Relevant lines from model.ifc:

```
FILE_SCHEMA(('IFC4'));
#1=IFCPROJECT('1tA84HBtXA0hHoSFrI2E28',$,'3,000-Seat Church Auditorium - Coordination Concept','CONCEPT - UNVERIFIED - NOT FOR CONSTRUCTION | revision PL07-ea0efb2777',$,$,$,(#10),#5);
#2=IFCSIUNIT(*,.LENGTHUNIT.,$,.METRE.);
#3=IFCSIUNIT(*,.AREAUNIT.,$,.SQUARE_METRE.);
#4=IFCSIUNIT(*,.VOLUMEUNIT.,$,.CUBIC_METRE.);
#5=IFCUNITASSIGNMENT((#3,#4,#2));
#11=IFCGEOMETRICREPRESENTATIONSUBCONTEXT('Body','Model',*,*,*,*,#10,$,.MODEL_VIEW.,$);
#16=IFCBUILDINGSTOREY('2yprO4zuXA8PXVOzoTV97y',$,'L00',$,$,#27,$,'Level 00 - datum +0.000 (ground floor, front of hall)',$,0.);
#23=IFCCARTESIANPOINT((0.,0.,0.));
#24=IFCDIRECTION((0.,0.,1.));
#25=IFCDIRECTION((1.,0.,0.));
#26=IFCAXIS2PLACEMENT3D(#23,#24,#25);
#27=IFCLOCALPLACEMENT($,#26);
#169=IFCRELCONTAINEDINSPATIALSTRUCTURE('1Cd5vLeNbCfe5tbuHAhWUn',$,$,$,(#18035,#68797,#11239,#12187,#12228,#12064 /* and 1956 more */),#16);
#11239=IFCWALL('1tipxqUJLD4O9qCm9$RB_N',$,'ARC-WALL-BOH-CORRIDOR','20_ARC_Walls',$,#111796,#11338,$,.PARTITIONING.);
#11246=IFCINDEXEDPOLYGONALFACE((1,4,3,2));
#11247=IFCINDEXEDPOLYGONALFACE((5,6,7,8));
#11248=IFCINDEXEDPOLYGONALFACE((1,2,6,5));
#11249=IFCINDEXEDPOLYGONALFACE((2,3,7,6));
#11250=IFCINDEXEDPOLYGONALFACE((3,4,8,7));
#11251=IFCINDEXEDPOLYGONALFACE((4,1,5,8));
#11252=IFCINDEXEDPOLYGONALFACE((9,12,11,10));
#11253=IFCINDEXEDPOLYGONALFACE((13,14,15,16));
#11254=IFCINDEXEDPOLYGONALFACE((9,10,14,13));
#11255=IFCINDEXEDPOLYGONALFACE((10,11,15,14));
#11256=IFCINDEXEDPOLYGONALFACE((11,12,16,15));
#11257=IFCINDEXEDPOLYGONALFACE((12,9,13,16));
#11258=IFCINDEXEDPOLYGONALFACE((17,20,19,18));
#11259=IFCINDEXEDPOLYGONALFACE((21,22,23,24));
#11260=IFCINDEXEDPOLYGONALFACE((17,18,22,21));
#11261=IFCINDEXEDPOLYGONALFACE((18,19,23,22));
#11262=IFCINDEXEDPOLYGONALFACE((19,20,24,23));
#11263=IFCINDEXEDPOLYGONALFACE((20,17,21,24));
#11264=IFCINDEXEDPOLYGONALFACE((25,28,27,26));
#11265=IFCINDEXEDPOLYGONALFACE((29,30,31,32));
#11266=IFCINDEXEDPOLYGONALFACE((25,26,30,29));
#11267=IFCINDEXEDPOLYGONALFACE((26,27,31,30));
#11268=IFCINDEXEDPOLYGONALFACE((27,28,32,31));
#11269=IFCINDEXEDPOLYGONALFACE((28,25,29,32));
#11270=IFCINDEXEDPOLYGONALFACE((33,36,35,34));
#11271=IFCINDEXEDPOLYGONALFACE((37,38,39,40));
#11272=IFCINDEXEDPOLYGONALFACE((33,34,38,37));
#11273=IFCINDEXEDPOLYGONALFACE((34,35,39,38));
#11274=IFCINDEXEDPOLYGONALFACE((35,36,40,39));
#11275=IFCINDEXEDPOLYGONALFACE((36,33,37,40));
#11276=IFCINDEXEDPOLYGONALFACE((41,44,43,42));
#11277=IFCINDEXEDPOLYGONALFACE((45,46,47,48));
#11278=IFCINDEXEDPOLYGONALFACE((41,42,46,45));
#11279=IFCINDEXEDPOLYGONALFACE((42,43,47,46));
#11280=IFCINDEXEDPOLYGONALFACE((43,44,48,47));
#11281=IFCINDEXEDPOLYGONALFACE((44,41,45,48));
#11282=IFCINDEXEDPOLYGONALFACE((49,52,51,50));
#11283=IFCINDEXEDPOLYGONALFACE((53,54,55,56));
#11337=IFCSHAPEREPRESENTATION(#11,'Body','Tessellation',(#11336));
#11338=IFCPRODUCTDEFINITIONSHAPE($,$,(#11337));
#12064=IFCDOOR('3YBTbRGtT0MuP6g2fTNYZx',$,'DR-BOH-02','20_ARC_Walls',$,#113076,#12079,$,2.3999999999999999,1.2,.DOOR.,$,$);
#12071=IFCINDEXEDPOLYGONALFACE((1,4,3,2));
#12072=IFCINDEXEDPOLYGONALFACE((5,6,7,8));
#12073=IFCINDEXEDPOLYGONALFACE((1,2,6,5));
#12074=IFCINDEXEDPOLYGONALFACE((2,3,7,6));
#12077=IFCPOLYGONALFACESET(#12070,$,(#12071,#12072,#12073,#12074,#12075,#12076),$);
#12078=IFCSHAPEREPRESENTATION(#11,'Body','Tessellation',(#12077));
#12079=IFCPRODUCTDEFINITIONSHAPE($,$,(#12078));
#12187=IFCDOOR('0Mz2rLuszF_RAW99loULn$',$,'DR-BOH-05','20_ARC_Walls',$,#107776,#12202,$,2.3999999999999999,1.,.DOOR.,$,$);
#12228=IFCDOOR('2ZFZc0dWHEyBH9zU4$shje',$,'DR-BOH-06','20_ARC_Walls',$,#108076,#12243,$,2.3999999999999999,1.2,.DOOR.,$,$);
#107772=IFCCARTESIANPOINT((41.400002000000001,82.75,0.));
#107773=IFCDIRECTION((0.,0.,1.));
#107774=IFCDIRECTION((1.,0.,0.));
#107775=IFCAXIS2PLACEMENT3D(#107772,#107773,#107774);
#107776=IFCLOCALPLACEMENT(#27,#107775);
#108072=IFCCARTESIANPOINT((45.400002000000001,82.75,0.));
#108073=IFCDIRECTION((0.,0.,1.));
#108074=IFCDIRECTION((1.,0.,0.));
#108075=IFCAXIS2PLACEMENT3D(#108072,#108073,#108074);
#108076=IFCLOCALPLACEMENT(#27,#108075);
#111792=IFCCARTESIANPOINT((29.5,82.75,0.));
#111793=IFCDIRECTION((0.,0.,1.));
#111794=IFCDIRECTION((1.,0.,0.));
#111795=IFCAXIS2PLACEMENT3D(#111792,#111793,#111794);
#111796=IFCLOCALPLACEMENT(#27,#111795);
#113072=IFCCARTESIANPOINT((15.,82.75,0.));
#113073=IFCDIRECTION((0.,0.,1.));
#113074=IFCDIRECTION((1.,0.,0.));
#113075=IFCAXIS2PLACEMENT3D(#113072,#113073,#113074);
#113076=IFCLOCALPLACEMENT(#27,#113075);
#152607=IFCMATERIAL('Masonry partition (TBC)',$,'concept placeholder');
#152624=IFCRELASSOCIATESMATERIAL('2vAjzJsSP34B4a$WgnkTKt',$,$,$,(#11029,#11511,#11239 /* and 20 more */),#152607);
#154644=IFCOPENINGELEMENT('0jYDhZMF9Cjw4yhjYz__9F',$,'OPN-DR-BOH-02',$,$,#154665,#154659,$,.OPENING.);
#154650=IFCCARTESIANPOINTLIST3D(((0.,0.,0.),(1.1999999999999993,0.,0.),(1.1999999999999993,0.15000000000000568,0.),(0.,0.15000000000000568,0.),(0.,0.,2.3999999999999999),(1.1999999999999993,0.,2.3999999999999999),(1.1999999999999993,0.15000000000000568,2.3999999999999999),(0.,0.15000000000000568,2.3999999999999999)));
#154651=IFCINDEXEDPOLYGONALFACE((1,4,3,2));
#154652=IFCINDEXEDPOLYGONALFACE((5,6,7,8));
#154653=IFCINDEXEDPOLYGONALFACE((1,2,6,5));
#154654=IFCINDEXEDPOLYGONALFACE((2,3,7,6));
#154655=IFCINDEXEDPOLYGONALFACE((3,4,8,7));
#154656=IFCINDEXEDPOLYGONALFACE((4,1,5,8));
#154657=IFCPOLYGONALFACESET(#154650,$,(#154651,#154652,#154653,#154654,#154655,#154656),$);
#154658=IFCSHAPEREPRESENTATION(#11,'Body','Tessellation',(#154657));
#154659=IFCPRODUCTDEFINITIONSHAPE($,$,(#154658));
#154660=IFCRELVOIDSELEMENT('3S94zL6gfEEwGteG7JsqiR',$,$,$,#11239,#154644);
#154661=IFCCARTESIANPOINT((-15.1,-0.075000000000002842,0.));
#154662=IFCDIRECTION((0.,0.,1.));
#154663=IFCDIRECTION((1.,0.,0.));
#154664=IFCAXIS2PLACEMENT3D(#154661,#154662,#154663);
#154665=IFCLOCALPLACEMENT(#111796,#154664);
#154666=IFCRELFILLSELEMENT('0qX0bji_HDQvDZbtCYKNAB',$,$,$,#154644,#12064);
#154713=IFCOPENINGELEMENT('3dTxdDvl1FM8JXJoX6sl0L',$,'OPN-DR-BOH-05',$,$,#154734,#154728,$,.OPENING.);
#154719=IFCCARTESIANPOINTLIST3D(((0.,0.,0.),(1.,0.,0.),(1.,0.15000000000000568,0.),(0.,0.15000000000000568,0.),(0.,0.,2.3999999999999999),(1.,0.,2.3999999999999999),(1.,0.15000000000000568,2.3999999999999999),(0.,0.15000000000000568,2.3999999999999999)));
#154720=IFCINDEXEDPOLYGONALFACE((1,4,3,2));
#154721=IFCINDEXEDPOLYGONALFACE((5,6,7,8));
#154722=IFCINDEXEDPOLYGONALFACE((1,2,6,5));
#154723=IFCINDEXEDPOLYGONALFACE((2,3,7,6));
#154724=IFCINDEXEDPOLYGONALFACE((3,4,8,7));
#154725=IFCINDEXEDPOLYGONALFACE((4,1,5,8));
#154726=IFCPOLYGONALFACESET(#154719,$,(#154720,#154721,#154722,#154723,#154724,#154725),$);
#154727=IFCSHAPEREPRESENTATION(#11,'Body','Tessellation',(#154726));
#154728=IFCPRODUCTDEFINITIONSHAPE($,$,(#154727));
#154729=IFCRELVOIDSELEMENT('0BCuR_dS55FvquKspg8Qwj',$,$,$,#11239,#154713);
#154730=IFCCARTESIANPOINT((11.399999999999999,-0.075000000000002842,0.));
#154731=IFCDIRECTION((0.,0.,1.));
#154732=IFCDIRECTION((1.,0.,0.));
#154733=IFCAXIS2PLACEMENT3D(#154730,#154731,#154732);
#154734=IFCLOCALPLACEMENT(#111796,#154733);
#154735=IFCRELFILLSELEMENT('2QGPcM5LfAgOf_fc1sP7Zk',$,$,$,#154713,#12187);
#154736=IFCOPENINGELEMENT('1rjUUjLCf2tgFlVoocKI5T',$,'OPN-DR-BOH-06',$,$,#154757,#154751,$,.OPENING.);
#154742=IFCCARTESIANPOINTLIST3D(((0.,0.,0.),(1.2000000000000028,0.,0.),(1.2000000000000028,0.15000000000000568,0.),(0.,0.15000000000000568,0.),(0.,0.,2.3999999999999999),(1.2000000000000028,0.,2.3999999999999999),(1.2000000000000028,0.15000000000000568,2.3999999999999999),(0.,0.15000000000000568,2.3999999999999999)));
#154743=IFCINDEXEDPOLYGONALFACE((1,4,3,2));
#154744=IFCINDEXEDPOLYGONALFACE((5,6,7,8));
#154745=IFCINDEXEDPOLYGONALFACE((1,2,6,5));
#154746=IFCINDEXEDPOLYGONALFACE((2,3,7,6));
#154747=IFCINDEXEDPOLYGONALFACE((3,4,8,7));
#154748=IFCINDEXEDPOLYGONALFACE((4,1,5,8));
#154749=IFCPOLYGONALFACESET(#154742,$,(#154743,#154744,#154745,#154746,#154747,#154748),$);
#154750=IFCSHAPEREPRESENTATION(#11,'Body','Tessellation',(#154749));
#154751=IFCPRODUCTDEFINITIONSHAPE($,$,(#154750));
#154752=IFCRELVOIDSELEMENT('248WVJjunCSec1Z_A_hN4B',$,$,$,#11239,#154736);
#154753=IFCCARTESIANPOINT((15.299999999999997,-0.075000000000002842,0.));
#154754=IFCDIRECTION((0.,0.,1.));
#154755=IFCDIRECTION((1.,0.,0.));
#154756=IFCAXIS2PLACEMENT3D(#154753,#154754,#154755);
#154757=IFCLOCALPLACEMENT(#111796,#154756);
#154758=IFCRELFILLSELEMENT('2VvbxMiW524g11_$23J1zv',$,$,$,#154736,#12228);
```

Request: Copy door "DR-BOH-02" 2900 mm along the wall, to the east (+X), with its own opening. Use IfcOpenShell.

```python
import ifcopenshell
import ifcopenshell.api.feature
import ifcopenshell.api.geometry
import ifcopenshell.api.root
import ifcopenshell.geom
import ifcopenshell.util.element
import ifcopenshell.util.placement
import ifcopenshell.util.shape
import ifcopenshell.util.unit

model = ifcopenshell.open("model.ifc")
unit_scale = ifcopenshell.util.unit.calculate_unit_scale(model)
settings = ifcopenshell.geom.settings()


def volume(element):
    """Net volume in cubic metres, openings subtracted."""
    shape = ifcopenshell.geom.create_shape(settings, element)
    return ifcopenshell.util.shape.get_volume(shape.geometry)


door = model.by_guid("3YBTbRGtT0MuP6g2fTNYZx")
opening = door.FillsVoids[0].RelatingOpeningElement
wall = opening.VoidsElements[0].RelatingBuildingElement
before = volume(wall)
shift = ifcopenshell.util.placement.get_local_placement(wall.ObjectPlacement)[:3, 0] * 2.9 / unit_scale

# copy_class copies the void relationship, type, container and properties, but no geometry.
new_opening = ifcopenshell.api.root.copy_class(model, product=opening)
new_opening.Representation = ifcopenshell.util.element.copy_deep(
    model, opening.Representation, exclude=["IfcGeometricRepresentationContext", "IfcRepresentationMap"]
)
new_door = ifcopenshell.api.root.copy_class(model, product=door)
new_door.Representation = ifcopenshell.util.element.copy_deep(
    model, door.Representation, exclude=["IfcGeometricRepresentationContext", "IfcRepresentationMap"]
)
ifcopenshell.api.feature.add_filling(model, opening=new_opening, element=new_door)

for old, new in ((opening, new_opening), (door, new_door)):
    matrix = ifcopenshell.util.placement.get_local_placement(old.ObjectPlacement)
    matrix[:3, 3] += shift
    ifcopenshell.api.geometry.edit_object_placement(model, product=new, matrix=matrix, is_si=False)

after = volume(wall)

print(f"wall volume {before:.3f} -> {after:.3f} m3")

model.write("model_updated.ifc")
```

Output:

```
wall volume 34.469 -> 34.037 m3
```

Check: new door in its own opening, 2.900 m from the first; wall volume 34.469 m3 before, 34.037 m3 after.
